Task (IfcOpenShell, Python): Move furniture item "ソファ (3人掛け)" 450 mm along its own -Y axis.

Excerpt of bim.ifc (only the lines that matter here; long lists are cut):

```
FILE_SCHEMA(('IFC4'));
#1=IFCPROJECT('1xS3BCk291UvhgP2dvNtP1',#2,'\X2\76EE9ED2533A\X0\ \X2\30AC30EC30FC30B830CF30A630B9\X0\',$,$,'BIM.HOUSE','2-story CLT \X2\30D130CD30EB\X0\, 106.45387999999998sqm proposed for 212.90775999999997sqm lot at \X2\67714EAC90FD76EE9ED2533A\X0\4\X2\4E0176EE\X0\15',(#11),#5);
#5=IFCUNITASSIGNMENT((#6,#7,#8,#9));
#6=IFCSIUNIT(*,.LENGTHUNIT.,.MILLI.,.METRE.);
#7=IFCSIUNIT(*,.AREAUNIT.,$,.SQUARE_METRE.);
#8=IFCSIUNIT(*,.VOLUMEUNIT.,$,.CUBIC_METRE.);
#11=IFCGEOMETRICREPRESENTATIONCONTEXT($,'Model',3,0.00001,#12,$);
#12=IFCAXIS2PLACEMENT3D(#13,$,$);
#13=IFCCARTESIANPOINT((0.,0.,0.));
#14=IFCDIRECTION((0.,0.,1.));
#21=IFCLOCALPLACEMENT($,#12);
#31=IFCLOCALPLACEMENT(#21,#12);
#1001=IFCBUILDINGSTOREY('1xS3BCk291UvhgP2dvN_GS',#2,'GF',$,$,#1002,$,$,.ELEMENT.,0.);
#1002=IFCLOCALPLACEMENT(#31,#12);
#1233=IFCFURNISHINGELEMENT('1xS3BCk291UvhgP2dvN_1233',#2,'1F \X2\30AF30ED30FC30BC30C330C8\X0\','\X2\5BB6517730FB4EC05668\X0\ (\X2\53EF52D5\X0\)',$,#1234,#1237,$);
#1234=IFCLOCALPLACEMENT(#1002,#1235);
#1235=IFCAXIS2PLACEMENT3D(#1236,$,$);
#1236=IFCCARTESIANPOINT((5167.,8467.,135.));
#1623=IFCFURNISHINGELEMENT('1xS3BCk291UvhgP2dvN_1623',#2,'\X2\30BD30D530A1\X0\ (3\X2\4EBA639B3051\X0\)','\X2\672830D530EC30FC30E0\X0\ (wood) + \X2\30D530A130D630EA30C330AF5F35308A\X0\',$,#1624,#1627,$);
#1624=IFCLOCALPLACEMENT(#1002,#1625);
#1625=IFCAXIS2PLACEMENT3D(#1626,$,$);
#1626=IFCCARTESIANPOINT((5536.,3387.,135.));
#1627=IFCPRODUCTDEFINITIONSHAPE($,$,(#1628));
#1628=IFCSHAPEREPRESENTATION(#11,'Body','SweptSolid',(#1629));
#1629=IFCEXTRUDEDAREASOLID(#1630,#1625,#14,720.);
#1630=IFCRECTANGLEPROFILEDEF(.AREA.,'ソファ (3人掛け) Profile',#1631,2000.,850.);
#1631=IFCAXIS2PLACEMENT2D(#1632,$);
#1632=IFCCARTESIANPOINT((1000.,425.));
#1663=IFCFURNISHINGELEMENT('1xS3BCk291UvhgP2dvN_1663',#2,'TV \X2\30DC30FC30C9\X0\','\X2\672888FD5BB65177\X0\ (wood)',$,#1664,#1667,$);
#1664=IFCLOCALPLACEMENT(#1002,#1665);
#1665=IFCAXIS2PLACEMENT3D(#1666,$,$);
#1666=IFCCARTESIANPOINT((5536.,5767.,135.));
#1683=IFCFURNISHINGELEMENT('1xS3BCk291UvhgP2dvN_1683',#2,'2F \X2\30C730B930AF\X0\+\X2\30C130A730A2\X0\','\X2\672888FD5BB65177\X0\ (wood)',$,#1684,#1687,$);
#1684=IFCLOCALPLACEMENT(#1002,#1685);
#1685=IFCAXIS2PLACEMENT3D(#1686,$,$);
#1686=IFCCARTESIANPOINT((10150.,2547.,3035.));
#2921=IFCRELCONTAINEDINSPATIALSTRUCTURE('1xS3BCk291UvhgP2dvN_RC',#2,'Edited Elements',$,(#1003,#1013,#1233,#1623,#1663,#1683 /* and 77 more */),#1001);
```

```python
import ifcopenshell
import ifcopenshell.api.geometry
import ifcopenshell.util.placement
import ifcopenshell.util.unit

model = ifcopenshell.open("bim.ifc")
unit_scale = ifcopenshell.util.unit.calculate_unit_scale(model)

item = model.by_guid("1xS3BCk291UvhgP2dvN_1623")
matrix = ifcopenshell.util.placement.get_local_placement(item.ObjectPlacement)
matrix[:3, 3] -= matrix[:3, 1] * 0.45 / unit_scale
ifcopenshell.api.geometry.edit_object_placement(model, product=item, matrix=matrix, is_si=False)

print(ifcopenshell.util.placement.get_local_placement(item.ObjectPlacement).round(3) + 0.0)

model.write("bim_updated.ifc")
```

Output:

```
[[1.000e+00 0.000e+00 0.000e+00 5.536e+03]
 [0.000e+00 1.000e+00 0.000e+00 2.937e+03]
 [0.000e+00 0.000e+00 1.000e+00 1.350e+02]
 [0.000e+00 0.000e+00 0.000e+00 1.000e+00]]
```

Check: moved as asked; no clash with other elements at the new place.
